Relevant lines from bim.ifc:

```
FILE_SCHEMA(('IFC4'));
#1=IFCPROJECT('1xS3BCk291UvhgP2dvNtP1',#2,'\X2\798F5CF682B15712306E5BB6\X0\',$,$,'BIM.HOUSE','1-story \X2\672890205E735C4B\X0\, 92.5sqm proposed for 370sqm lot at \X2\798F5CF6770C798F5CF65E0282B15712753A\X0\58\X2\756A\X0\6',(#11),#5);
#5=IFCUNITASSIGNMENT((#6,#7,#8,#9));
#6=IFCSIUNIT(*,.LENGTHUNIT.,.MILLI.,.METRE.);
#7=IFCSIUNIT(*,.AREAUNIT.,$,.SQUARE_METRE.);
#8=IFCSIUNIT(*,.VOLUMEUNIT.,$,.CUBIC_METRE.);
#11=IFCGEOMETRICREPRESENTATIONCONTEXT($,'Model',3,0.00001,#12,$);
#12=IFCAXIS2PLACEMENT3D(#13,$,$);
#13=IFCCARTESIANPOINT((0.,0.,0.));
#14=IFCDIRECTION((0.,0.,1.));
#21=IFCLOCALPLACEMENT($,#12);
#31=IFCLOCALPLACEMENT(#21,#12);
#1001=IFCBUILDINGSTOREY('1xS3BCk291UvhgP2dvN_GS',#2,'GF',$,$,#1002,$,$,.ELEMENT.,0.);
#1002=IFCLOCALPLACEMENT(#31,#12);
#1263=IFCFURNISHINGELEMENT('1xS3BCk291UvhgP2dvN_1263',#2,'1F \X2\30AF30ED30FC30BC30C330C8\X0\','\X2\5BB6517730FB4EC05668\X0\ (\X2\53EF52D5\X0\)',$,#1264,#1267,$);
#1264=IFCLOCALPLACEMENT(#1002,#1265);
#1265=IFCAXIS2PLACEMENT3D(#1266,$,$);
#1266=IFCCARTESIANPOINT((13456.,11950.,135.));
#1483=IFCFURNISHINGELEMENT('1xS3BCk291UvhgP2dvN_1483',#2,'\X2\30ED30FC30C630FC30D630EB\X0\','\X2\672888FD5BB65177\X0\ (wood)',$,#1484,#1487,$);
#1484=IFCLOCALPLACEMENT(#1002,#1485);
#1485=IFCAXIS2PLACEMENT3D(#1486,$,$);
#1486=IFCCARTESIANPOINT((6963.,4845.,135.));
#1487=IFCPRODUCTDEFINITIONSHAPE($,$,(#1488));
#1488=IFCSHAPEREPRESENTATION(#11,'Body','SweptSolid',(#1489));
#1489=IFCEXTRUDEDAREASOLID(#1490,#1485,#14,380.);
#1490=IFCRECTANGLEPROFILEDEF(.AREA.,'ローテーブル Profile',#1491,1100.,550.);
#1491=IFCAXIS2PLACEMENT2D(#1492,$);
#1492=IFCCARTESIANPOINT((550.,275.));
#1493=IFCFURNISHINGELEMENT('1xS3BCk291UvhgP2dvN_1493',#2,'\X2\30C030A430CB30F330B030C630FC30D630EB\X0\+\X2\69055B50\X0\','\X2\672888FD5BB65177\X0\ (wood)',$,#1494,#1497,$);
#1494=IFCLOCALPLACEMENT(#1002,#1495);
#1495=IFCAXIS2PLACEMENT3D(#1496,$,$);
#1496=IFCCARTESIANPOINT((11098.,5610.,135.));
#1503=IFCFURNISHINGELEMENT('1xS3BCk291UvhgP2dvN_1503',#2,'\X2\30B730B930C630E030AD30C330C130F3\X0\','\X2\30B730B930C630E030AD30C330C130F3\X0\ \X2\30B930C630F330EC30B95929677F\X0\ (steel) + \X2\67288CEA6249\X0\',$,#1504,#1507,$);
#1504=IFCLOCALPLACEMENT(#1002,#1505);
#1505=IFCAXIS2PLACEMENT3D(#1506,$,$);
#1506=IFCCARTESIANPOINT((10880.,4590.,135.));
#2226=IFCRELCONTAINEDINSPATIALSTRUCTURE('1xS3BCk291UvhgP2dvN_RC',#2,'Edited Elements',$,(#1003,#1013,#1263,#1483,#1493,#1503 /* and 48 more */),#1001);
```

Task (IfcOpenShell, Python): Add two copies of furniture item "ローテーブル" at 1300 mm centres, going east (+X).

```python
import numpy as np
import ifcopenshell
import ifcopenshell.api.geometry
import ifcopenshell.api.root
import ifcopenshell.util.element
import ifcopenshell.util.placement
import ifcopenshell.util.unit

model = ifcopenshell.open("bim.ifc")
unit_scale = ifcopenshell.util.unit.calculate_unit_scale(model)


def reuse_history(source, copy):
    """copy_class also copies each property set's owner history, people and application; keep the originals."""
    for rel in copy.IsDefinedBy:
        if rel.is_a("IfcRelDefinesByProperties") and (history := rel.RelatingPropertyDefinition.OwnerHistory):
            rel.RelatingPropertyDefinition.OwnerHistory = source.OwnerHistory
            ifcopenshell.util.element.remove_deep2(model, history)


source = model.by_id(1483)
base = ifcopenshell.util.placement.get_local_placement(source.ObjectPlacement)
step = np.array([1.0, 0.0, 0.0]) * 1.3 / unit_scale

for i in range(1, 3):
    copy = ifcopenshell.api.root.copy_class(model, product=source)
    copy.Representation = ifcopenshell.util.element.copy_deep(
        model, source.Representation, exclude=["IfcGeometricRepresentationContext", "IfcRepresentationMap"]
    )
    reuse_history(source, copy)
    matrix = base.copy()
    matrix[:3, 3] += i * step
    print("added at", matrix[:3, 3].round(3) + 0.0)
    ifcopenshell.api.geometry.edit_object_placement(model, product=copy, matrix=matrix, is_si=False)

model.write("bim-out.ifc")
```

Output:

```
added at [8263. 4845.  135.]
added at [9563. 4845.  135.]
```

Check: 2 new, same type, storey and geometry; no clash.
